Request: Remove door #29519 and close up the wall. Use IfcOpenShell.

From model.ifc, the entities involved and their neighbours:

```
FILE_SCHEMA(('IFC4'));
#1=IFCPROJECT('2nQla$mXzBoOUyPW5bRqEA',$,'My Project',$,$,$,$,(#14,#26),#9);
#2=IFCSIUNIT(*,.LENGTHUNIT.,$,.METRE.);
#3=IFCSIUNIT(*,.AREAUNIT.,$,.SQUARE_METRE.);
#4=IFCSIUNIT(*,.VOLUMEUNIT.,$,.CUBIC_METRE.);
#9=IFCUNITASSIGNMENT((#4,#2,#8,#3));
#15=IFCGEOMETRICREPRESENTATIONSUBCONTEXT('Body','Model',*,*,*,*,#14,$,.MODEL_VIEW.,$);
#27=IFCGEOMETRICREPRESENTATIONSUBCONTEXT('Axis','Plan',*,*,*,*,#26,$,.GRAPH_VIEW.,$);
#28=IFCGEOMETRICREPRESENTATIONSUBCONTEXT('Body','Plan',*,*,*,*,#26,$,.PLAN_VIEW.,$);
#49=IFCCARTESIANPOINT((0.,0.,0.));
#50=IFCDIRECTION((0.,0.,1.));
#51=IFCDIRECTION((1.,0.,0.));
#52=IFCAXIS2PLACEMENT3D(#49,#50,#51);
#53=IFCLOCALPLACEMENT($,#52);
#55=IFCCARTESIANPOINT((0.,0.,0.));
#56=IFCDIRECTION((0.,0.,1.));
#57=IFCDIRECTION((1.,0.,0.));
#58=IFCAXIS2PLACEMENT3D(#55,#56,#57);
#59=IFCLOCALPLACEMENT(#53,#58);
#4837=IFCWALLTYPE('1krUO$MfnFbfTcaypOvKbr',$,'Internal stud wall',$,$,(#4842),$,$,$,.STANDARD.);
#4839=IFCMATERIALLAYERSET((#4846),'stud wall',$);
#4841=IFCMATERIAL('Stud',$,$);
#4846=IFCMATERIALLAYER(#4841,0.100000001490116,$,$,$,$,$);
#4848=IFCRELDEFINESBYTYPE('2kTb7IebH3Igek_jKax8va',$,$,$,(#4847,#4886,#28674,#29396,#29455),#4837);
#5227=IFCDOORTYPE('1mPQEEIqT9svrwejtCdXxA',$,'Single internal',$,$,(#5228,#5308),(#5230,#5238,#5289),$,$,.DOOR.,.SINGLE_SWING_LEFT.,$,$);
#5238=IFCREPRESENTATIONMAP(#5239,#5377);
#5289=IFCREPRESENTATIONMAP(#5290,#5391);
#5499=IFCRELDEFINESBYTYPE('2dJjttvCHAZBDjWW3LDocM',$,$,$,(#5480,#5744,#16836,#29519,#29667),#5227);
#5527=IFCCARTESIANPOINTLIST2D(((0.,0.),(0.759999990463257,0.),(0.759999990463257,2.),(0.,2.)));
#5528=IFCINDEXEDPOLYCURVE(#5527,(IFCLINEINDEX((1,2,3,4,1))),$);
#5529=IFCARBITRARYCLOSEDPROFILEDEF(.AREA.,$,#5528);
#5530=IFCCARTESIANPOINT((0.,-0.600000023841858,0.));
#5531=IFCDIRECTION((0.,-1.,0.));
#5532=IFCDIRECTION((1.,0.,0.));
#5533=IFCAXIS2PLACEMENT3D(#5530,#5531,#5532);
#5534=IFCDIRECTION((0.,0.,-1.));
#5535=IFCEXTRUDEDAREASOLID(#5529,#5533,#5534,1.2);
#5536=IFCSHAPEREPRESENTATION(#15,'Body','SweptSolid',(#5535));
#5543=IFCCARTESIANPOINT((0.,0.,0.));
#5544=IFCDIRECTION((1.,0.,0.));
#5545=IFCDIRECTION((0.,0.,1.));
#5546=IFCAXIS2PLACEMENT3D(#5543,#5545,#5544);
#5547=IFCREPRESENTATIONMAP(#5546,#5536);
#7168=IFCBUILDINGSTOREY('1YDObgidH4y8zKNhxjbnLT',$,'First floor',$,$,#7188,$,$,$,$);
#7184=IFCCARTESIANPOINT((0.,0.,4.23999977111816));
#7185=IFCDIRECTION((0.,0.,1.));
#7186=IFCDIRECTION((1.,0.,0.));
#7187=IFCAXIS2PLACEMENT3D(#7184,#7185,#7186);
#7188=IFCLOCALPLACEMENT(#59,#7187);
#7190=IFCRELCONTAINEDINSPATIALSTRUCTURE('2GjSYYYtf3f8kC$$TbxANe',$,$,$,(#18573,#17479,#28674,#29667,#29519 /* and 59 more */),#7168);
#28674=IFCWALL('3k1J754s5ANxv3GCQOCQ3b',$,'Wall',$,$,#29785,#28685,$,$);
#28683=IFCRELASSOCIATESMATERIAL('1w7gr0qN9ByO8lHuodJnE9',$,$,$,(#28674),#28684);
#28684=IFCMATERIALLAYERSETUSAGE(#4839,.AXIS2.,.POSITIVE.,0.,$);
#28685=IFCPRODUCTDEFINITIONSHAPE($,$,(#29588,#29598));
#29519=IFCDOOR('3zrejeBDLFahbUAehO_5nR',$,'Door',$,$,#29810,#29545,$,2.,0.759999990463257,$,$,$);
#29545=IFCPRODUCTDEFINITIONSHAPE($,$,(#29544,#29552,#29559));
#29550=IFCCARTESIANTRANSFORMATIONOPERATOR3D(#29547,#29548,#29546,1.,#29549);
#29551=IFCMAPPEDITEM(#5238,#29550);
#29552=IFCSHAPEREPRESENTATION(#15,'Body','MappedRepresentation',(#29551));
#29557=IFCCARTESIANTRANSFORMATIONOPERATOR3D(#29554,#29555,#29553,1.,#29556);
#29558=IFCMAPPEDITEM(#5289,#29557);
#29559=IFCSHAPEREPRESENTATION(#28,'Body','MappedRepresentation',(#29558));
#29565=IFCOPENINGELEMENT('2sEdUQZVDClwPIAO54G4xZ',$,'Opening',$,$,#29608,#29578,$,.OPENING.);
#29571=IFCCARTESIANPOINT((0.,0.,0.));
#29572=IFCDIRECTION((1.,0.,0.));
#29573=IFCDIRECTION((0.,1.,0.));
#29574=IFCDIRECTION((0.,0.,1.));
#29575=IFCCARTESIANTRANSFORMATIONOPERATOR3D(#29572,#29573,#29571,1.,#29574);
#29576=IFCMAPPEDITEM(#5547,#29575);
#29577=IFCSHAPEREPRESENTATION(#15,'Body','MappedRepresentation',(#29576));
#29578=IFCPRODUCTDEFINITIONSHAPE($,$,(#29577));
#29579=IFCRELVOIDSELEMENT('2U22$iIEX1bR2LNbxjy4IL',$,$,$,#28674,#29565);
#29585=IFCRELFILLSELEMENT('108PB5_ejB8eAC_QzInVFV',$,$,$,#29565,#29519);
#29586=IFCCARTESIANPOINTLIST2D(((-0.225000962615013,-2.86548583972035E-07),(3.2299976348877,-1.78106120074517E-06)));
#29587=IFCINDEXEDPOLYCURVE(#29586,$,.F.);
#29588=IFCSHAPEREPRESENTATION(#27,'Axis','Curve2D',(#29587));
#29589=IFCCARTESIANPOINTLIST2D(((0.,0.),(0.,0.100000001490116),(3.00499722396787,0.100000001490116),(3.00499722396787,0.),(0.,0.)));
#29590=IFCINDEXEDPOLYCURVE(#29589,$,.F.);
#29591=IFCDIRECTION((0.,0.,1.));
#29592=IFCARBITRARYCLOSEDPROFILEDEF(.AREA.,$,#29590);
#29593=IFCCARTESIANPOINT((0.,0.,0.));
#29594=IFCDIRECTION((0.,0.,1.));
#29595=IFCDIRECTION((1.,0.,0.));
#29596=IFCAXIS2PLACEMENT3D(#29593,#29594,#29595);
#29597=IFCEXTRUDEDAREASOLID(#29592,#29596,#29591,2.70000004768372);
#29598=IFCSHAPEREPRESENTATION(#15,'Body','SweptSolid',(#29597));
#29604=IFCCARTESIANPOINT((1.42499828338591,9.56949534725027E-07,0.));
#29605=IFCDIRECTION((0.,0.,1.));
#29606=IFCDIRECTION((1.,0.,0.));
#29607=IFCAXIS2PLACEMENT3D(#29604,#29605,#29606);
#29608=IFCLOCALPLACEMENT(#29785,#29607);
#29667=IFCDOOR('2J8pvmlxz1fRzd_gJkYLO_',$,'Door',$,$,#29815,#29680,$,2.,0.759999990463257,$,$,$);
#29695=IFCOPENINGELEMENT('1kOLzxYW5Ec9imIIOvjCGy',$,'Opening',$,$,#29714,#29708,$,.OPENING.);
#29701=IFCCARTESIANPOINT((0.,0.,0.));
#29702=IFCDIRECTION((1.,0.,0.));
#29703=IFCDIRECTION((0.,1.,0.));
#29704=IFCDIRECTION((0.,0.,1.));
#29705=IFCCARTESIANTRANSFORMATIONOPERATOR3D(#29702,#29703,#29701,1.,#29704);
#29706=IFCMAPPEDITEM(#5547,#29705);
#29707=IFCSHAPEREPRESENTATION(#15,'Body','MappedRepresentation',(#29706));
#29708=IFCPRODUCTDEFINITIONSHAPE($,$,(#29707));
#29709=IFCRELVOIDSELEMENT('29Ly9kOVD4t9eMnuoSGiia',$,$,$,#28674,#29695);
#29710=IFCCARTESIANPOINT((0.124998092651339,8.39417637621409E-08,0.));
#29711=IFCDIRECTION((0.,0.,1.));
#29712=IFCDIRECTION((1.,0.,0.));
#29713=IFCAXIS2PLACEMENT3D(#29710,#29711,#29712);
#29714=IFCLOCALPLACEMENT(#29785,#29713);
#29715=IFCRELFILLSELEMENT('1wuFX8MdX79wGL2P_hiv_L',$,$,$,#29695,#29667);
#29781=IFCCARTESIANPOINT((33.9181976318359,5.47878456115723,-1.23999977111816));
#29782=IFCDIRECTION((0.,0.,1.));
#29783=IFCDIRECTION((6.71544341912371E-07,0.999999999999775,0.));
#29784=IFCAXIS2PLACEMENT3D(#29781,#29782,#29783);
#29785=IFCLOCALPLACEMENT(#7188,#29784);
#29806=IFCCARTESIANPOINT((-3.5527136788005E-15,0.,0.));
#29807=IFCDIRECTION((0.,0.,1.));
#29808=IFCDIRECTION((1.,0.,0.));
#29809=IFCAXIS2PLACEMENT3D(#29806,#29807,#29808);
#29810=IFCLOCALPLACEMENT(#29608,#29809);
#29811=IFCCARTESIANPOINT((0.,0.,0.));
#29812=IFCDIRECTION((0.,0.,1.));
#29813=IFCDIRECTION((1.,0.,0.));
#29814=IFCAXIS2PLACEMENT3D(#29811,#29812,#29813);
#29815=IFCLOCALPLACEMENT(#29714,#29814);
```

```python
import ifcopenshell
import ifcopenshell.api.feature
import ifcopenshell.api.root
import ifcopenshell.geom
import ifcopenshell.util.shape

model = ifcopenshell.open("model.ifc")
settings = ifcopenshell.geom.settings()


def volume(element):
    """Net volume in cubic metres, openings subtracted."""
    shape = ifcopenshell.geom.create_shape(settings, element)
    return ifcopenshell.util.shape.get_volume(shape.geometry)


door = model.by_id(29519)
opening = door.FillsVoids[0].RelatingOpeningElement
wall = opening.VoidsElements[0].RelatingBuildingElement
before = volume(wall)

ifcopenshell.api.root.remove_product(model, product=door)
ifcopenshell.api.feature.remove_feature(model, feature=opening)

after = volume(wall)

print(f"wall volume {before:.3f} -> {after:.3f} m3")

model.write("model_edited.ifc")
```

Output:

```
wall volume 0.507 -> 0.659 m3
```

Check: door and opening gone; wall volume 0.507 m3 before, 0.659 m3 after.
